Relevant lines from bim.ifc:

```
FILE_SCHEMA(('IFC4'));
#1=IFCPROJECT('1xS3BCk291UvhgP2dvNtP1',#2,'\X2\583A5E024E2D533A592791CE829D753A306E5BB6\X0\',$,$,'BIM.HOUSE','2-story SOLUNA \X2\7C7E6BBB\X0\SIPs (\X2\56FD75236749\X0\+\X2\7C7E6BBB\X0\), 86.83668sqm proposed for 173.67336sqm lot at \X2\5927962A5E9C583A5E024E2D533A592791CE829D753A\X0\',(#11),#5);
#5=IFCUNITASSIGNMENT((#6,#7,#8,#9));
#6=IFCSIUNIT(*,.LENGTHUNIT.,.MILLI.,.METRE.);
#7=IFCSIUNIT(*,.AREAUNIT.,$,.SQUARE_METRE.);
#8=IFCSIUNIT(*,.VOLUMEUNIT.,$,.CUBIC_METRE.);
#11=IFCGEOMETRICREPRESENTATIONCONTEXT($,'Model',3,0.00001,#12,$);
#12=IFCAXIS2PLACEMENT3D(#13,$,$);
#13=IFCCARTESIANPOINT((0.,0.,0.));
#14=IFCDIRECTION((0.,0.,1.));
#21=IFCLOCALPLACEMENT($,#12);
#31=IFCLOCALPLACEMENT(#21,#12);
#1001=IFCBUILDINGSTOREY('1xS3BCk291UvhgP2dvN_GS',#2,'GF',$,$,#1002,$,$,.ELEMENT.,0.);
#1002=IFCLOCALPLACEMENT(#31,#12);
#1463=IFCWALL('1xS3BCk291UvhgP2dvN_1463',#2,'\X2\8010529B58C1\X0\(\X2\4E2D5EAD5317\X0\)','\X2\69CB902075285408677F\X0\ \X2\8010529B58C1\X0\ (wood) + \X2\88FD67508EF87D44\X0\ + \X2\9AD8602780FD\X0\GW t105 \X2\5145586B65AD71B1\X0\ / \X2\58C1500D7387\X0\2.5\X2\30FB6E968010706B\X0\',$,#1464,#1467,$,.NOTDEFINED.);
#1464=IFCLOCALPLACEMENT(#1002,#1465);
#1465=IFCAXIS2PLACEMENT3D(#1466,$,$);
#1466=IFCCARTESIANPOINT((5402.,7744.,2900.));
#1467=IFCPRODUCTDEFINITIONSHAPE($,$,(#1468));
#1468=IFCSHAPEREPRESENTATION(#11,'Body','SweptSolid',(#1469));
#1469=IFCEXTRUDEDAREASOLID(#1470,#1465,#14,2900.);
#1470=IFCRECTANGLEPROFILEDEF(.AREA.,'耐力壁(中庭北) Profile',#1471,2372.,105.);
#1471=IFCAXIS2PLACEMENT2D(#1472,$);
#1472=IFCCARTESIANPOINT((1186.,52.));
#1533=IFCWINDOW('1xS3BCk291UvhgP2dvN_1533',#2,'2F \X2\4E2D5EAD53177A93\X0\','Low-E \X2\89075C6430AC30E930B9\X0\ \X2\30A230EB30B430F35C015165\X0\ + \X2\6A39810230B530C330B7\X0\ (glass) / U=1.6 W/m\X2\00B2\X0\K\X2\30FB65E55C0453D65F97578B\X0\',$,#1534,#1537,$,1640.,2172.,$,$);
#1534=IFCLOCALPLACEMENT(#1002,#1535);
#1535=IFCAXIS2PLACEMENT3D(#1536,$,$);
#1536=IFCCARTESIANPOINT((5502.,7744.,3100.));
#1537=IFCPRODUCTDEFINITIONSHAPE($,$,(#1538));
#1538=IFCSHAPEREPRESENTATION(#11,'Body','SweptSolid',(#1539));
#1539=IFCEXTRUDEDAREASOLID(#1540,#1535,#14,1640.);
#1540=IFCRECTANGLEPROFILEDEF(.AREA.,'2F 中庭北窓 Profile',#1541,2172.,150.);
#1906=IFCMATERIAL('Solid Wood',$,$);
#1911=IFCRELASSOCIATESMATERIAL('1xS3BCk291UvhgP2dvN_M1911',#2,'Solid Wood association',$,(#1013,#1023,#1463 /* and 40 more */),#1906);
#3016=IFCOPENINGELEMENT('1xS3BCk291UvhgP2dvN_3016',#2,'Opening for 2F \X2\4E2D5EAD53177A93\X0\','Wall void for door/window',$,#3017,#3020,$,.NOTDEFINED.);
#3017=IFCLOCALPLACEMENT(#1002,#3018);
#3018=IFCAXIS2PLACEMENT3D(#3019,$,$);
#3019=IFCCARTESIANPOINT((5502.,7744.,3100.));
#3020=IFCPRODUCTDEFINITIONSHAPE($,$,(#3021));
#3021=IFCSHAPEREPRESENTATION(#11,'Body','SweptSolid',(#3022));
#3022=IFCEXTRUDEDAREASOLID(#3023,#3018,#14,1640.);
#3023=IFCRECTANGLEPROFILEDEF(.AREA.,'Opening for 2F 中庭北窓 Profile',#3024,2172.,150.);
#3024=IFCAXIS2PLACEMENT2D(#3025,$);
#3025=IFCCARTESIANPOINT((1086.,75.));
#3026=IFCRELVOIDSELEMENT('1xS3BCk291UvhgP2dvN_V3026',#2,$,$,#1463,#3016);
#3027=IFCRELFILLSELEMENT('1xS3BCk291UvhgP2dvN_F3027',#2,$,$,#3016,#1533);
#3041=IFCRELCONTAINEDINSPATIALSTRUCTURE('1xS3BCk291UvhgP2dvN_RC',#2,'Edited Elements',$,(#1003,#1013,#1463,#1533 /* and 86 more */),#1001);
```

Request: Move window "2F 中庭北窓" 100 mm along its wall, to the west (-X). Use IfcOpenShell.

```python
import ifcopenshell
import ifcopenshell.api.geometry
import ifcopenshell.util.placement

model = ifcopenshell.open("bim.ifc")

window = model.by_guid("1xS3BCk291UvhgP2dvN_1533")
opening = window.FillsVoids[0].RelatingOpeningElement
wall = opening.VoidsElements[0].RelatingBuildingElement

wall_matrix = ifcopenshell.util.placement.get_local_placement(wall.ObjectPlacement)
shift = wall_matrix[:3, 0] * -100.0
before = ifcopenshell.util.placement.get_local_placement(window.ObjectPlacement)[:3, 3].copy()

# The window is not placed relative to its opening, so move both.
for product in (opening, window):
    matrix = ifcopenshell.util.placement.get_local_placement(product.ObjectPlacement)
    matrix[:3, 3] += shift
    ifcopenshell.api.geometry.edit_object_placement(model, product=product, matrix=matrix, is_si=False)

after = ifcopenshell.util.placement.get_local_placement(window.ObjectPlacement)[:3, 3]
print("window moved by", (after - before).round(3) + 0.0)

model.write("bim-out.ifc")
```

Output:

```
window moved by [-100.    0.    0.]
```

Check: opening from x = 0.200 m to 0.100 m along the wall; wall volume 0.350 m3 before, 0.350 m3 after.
